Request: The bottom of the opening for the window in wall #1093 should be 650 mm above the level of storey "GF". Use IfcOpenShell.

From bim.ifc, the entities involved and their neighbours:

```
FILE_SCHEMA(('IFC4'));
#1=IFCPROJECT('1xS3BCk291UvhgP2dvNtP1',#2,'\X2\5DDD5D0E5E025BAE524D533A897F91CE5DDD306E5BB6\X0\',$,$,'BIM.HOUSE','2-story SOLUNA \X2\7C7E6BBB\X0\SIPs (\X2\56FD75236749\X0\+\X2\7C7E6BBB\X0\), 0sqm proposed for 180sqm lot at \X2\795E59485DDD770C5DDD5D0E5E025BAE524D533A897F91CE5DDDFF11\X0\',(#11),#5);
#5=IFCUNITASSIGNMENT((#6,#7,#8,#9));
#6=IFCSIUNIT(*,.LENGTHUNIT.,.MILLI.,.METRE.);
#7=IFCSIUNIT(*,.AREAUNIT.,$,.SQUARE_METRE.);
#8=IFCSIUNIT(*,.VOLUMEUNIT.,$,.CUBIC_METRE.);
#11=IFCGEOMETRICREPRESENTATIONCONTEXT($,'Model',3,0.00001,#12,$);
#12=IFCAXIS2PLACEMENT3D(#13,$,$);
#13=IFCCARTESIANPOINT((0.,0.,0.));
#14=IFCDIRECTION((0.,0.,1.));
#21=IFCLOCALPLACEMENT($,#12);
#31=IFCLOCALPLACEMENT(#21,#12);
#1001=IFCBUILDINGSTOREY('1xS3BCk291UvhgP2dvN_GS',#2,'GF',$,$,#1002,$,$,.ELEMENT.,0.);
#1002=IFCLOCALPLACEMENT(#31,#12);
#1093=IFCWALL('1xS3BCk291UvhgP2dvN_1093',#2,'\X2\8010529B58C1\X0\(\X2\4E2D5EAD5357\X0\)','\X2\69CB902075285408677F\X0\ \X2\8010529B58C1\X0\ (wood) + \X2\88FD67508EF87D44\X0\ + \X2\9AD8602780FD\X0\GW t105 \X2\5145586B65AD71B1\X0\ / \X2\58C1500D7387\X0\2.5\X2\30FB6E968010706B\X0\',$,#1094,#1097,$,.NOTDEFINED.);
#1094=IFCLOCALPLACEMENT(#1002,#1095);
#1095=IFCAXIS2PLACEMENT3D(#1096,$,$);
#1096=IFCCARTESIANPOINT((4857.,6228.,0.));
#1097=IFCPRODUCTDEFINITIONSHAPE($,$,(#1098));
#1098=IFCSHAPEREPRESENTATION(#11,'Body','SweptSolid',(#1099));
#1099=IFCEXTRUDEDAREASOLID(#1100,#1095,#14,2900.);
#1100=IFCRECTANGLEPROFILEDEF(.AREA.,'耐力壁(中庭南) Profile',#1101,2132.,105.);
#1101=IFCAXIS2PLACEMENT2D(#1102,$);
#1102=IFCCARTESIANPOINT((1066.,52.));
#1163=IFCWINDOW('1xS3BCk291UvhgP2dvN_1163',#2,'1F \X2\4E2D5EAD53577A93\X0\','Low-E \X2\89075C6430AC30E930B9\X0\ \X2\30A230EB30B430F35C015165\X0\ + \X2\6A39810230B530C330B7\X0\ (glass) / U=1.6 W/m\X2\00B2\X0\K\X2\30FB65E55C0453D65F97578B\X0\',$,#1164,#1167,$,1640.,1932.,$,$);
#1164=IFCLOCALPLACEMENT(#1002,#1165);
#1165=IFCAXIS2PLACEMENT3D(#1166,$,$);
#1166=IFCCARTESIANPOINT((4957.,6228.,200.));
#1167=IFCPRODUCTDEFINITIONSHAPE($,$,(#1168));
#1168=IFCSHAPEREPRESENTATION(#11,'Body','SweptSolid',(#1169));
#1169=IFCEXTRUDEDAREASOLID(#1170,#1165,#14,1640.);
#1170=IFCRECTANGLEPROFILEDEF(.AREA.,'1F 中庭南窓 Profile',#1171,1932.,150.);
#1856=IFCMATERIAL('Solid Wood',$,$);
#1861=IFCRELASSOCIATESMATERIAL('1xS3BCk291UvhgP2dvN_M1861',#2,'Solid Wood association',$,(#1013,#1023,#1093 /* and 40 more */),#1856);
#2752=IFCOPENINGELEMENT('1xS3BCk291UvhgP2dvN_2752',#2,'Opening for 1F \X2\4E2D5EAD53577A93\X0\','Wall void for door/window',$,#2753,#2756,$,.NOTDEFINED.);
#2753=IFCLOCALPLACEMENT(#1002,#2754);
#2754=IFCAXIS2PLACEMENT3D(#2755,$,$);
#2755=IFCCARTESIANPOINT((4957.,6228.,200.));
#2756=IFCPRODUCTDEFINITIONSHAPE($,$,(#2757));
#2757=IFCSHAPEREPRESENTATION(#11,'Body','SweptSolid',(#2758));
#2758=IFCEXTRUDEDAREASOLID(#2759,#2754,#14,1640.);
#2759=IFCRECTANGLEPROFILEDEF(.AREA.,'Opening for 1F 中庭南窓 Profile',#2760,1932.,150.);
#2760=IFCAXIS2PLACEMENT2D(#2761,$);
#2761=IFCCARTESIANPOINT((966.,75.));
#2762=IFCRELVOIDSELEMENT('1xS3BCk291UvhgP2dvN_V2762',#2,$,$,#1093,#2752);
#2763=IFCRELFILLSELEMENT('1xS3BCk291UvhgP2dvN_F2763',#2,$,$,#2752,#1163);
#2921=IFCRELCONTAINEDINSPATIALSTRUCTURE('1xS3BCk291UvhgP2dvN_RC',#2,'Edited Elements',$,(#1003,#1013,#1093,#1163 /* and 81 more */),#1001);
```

```python
import numpy as np
import ifcopenshell
import ifcopenshell.api.geometry
import ifcopenshell.geom
import ifcopenshell.util.element
import ifcopenshell.util.placement
import ifcopenshell.util.shape
import ifcopenshell.util.unit

model = ifcopenshell.open("bim.ifc")
unit_scale = ifcopenshell.util.unit.calculate_unit_scale(model)

window = model.by_id(1163)
opening = window.FillsVoids[0].RelatingOpeningElement
storey = ifcopenshell.util.element.get_container(window, ifc_class="IfcBuildingStorey")
level = ifcopenshell.util.placement.get_local_placement(storey.ObjectPlacement)[2, 3]

# The opening's origin need not be at the sill, so measure its lowest point.
shape = ifcopenshell.geom.create_shape(ifcopenshell.geom.settings(), opening)
bottom = ifcopenshell.util.shape.get_shape_bottom_elevation(shape, shape.geometry) / unit_scale
dz = level + 0.65 / unit_scale - bottom

shift = np.array([0.0, 0.0, dz])
# The window is not placed relative to its opening, so move both.
for product in (opening, window):
    matrix = ifcopenshell.util.placement.get_local_placement(product.ObjectPlacement)
    matrix[:3, 3] += shift
    ifcopenshell.api.geometry.edit_object_placement(model, product=product, matrix=matrix, is_si=False)

print(f"moved by {dz * unit_scale:+.3f} m")

model.write("bim_edited.ifc")
```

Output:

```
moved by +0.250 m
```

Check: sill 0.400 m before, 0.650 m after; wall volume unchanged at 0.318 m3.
